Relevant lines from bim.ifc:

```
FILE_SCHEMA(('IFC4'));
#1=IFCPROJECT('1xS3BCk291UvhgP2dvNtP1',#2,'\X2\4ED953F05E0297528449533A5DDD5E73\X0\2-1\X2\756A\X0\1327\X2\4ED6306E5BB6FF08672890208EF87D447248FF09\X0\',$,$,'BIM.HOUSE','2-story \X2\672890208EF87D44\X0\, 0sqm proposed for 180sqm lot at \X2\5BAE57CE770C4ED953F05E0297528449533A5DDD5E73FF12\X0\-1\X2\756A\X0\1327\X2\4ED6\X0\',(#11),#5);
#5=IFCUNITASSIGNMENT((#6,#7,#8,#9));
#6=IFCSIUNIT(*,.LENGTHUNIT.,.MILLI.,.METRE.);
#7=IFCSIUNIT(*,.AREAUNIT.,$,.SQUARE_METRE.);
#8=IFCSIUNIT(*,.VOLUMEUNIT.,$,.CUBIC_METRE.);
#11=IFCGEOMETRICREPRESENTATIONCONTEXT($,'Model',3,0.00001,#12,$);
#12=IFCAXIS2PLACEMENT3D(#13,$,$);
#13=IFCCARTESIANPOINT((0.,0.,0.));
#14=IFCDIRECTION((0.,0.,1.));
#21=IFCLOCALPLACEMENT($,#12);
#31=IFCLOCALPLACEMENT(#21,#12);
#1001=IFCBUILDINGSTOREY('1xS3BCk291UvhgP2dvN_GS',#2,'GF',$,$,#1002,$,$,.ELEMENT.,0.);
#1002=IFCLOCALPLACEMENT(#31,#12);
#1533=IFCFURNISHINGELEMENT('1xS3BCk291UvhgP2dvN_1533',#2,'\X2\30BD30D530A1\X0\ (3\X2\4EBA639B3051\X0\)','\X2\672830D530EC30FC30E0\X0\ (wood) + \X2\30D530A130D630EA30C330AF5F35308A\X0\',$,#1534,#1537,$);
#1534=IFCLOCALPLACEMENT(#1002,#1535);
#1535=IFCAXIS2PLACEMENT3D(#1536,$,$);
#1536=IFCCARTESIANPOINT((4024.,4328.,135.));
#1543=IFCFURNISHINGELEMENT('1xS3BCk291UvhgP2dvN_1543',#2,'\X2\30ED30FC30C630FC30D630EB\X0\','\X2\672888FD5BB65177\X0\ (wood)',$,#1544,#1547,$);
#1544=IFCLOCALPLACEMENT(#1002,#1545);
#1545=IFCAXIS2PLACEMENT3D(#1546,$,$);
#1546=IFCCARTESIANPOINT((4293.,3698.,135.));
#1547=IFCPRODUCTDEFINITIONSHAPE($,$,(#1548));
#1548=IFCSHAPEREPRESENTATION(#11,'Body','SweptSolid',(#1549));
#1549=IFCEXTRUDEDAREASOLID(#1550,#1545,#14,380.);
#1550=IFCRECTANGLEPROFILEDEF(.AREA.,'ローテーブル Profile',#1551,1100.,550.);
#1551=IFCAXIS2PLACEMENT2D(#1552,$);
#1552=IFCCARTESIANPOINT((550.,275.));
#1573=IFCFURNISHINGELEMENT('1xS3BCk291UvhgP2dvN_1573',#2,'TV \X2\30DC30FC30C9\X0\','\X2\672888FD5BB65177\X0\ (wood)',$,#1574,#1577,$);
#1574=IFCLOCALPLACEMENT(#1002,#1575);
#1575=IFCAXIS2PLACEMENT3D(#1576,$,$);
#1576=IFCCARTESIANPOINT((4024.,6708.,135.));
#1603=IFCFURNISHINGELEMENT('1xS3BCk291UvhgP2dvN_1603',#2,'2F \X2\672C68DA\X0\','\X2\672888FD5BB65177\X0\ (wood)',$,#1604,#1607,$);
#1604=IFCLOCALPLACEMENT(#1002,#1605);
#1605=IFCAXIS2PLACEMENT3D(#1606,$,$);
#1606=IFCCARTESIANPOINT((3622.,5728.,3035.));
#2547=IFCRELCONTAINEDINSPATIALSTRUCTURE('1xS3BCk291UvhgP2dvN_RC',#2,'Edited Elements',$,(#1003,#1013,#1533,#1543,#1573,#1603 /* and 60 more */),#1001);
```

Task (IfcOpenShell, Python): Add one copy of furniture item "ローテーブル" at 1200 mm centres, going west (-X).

```python
import numpy as np
import ifcopenshell
import ifcopenshell.api.geometry
import ifcopenshell.api.root
import ifcopenshell.util.element
import ifcopenshell.util.placement
import ifcopenshell.util.unit

model = ifcopenshell.open("bim.ifc")
unit_scale = ifcopenshell.util.unit.calculate_unit_scale(model)


def reuse_history(source, copy):
    """copy_class also copies each property set's owner history, people and application; keep the originals."""
    for rel in copy.IsDefinedBy:
        if rel.is_a("IfcRelDefinesByProperties") and (history := rel.RelatingPropertyDefinition.OwnerHistory):
            rel.RelatingPropertyDefinition.OwnerHistory = source.OwnerHistory
            ifcopenshell.util.element.remove_deep2(model, history)


source = model.by_guid("1xS3BCk291UvhgP2dvN_1543")
base = ifcopenshell.util.placement.get_local_placement(source.ObjectPlacement)
step = np.array([-1.0, 0.0, 0.0]) * 1.2 / unit_scale

for i in range(1, 2):
    copy = ifcopenshell.api.root.copy_class(model, product=source)
    copy.Representation = ifcopenshell.util.element.copy_deep(
        model, source.Representation, exclude=["IfcGeometricRepresentationContext", "IfcRepresentationMap"]
    )
    reuse_history(source, copy)
    matrix = base.copy()
    matrix[:3, 3] += i * step
    print("added at", matrix[:3, 3].round(3) + 0.0)
    ifcopenshell.api.geometry.edit_object_placement(model, product=copy, matrix=matrix, is_si=False)

model.write("bim_v2.ifc")
```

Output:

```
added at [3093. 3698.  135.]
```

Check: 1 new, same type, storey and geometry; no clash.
